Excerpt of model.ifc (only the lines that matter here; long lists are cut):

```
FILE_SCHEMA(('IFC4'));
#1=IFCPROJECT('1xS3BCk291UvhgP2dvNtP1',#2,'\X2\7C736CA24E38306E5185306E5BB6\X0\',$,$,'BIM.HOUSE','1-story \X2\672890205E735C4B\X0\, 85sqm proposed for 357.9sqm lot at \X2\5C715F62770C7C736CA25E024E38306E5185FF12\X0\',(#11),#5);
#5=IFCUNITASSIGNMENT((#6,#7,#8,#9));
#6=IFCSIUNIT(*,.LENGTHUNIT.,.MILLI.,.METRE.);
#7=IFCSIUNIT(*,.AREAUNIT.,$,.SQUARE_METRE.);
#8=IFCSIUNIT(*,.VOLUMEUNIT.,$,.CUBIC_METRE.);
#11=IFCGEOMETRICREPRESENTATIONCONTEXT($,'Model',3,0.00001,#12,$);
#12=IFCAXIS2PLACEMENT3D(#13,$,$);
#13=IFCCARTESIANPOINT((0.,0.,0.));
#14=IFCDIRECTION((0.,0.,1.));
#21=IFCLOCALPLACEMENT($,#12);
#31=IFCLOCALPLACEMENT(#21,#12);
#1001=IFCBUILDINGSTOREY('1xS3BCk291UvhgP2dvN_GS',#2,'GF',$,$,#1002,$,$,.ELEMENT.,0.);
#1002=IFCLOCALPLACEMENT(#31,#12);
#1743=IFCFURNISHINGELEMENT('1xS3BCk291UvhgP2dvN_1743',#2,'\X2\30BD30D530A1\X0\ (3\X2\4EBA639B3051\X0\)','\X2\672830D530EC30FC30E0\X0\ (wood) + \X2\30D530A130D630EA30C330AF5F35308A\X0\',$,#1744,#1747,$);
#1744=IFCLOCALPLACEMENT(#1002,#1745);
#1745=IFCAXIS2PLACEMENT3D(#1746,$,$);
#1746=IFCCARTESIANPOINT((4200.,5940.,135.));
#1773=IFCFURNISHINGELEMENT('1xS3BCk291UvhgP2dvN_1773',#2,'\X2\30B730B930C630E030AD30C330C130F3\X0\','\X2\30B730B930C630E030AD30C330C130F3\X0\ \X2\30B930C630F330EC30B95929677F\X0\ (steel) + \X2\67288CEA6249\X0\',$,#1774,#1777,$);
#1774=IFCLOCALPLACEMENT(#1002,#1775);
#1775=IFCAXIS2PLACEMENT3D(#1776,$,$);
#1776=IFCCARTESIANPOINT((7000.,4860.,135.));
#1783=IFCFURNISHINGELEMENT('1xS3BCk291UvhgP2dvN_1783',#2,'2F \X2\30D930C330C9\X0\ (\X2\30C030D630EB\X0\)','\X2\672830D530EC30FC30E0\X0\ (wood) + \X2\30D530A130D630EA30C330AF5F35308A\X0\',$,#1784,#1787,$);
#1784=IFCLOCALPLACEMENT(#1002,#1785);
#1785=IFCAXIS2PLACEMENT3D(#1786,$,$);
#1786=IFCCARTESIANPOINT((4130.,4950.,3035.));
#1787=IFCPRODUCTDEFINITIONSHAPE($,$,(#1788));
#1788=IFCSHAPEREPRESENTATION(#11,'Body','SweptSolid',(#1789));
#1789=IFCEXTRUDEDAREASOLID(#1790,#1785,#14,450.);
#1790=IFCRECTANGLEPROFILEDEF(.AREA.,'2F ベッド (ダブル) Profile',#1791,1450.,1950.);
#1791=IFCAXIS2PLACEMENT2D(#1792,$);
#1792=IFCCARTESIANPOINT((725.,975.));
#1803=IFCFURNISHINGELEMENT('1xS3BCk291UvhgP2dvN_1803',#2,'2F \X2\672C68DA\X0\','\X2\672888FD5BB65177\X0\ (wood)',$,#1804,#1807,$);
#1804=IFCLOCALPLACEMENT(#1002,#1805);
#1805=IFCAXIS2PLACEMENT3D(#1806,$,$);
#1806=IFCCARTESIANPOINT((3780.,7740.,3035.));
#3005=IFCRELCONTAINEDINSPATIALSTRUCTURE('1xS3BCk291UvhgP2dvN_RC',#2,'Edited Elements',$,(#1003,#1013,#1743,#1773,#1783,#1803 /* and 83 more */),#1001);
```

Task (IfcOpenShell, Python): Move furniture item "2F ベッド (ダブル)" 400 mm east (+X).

```python
import ifcopenshell
import ifcopenshell.api.geometry
import ifcopenshell.util.placement
import ifcopenshell.util.unit

model = ifcopenshell.open("model.ifc")
unit_scale = ifcopenshell.util.unit.calculate_unit_scale(model)

item = model.by_id(1783)
matrix = ifcopenshell.util.placement.get_local_placement(item.ObjectPlacement)
matrix[0, 3] += 0.4 / unit_scale
ifcopenshell.api.geometry.edit_object_placement(model, product=item, matrix=matrix, is_si=False)

print(ifcopenshell.util.placement.get_local_placement(item.ObjectPlacement).round(3) + 0.0)

model.write("model_updated.ifc")
```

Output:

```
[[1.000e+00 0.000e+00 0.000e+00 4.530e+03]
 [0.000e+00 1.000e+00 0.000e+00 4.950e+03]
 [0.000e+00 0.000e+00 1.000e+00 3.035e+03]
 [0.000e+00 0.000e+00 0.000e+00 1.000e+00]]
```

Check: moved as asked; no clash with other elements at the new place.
